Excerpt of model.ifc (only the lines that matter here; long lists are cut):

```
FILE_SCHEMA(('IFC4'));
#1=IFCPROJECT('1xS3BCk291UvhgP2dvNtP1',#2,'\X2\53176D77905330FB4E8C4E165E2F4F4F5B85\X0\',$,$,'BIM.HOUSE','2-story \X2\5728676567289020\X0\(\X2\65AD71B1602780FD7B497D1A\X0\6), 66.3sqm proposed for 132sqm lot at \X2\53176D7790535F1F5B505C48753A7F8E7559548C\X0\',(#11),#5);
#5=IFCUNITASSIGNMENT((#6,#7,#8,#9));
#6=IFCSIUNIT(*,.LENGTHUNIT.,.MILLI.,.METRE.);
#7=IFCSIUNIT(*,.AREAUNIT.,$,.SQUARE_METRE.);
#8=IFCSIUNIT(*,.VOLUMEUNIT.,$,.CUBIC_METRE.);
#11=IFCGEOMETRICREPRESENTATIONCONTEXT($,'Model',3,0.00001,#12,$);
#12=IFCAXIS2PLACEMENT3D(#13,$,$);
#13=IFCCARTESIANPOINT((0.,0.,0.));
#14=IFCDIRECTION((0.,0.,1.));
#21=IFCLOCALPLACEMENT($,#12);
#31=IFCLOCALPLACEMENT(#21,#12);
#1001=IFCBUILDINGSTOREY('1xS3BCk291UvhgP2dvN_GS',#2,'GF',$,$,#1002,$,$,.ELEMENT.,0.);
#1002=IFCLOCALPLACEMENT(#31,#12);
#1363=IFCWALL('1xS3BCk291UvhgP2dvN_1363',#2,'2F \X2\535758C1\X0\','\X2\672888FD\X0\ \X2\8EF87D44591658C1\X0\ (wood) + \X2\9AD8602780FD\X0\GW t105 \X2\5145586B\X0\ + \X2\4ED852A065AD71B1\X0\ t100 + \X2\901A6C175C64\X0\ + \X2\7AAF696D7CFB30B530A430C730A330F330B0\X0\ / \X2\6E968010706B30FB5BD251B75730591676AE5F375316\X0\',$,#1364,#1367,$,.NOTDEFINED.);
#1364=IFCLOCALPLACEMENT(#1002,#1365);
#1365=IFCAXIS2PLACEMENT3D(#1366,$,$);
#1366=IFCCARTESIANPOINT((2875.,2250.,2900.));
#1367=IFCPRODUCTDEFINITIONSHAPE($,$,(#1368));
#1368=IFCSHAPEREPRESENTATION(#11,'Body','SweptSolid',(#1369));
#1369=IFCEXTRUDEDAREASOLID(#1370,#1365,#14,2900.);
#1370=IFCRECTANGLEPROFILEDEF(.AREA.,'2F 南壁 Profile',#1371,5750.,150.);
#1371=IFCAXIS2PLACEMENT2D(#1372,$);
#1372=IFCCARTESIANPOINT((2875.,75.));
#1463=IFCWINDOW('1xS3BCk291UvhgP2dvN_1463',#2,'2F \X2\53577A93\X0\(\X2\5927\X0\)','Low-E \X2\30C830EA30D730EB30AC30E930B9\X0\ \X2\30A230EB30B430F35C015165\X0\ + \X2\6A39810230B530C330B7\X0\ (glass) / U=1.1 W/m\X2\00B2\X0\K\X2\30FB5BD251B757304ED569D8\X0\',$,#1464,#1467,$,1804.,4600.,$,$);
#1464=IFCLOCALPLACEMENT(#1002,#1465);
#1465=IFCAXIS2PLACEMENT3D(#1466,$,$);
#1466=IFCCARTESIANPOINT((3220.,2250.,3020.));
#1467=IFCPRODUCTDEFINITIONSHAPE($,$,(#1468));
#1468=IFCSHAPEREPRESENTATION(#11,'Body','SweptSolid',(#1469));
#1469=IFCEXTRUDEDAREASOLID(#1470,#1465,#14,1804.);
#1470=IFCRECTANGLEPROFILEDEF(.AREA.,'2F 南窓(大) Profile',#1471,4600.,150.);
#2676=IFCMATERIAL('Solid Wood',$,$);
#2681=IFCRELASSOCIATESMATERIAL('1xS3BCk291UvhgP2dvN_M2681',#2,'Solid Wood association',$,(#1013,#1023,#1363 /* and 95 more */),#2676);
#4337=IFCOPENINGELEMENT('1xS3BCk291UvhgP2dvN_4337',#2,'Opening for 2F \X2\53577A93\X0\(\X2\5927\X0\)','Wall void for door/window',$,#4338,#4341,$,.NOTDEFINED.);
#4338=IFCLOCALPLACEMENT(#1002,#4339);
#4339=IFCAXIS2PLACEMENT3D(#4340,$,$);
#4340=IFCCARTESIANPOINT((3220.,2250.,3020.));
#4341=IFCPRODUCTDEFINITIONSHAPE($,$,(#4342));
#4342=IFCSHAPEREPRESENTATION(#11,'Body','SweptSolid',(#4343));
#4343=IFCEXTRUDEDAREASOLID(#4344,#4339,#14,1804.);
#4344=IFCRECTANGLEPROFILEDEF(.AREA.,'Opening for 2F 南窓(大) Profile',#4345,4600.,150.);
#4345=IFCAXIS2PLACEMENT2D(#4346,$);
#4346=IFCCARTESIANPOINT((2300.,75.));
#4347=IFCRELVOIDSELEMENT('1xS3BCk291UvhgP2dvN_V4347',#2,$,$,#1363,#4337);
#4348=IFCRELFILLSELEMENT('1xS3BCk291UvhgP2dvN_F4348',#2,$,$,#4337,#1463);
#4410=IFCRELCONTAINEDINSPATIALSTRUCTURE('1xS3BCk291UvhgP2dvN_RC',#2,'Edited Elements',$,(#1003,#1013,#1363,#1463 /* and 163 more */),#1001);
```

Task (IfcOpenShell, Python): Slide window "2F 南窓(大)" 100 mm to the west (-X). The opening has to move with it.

```python
import ifcopenshell
import ifcopenshell.api.geometry
import ifcopenshell.util.placement
import ifcopenshell.util.unit

model = ifcopenshell.open("model.ifc")
unit_scale = ifcopenshell.util.unit.calculate_unit_scale(model)

window = model.by_guid("1xS3BCk291UvhgP2dvN_1463")
opening = window.FillsVoids[0].RelatingOpeningElement
wall = opening.VoidsElements[0].RelatingBuildingElement

wall_matrix = ifcopenshell.util.placement.get_local_placement(wall.ObjectPlacement)
shift = wall_matrix[:3, 0] * -0.1 / unit_scale
before = ifcopenshell.util.placement.get_local_placement(window.ObjectPlacement)[:3, 3].copy()

# The window is not placed relative to its opening, so move both.
for product in (opening, window):
    matrix = ifcopenshell.util.placement.get_local_placement(product.ObjectPlacement)
    matrix[:3, 3] += shift
    ifcopenshell.api.geometry.edit_object_placement(model, product=product, matrix=matrix, is_si=False)

after = ifcopenshell.util.placement.get_local_placement(window.ObjectPlacement)[:3, 3]
print("window moved by", (after - before).round(3) + 0.0)

model.write("model_rev.ifc")
```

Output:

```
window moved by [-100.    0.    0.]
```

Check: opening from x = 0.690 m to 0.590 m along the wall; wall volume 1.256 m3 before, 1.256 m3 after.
